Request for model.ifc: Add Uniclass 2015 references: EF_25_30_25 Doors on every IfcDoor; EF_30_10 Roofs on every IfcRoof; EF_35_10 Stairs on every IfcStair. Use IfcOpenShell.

First a look at what the model holds.

```python
import ifcopenshell

model = ifcopenshell.open("model.ifc")
print(model.schema)
print("classifications:", [c.Name for c in model.by_type("IfcClassification")])
for ifc_class in ("IfcDoor", "IfcRoof", "IfcStair", "IfcWall", "IfcWindow"):
    print(ifc_class, len(model.by_type(ifc_class)))
```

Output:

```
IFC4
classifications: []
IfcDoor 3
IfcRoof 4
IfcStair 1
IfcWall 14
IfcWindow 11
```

```python
import ifcopenshell
import ifcopenshell.api.classification

model = ifcopenshell.open("model.ifc")

system = ifcopenshell.api.classification.add_classification(model, classification="Uniclass 2015")

codes = {
    "IfcDoor": ("EF_25_30_25", "Doors"),
    "IfcRoof": ("EF_30_10", "Roofs"),
    "IfcStair": ("EF_35_10", "Stairs"),
}
for ifc_class, (code, name) in codes.items():
    products = model.by_type(ifc_class)
    ifcopenshell.api.classification.add_reference(
        model, products=products, classification=system, identification=code, name=name
    )
    print(code, len(products))

model.write("model_v2.ifc")
```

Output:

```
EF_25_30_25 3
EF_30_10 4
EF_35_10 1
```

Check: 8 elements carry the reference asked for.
